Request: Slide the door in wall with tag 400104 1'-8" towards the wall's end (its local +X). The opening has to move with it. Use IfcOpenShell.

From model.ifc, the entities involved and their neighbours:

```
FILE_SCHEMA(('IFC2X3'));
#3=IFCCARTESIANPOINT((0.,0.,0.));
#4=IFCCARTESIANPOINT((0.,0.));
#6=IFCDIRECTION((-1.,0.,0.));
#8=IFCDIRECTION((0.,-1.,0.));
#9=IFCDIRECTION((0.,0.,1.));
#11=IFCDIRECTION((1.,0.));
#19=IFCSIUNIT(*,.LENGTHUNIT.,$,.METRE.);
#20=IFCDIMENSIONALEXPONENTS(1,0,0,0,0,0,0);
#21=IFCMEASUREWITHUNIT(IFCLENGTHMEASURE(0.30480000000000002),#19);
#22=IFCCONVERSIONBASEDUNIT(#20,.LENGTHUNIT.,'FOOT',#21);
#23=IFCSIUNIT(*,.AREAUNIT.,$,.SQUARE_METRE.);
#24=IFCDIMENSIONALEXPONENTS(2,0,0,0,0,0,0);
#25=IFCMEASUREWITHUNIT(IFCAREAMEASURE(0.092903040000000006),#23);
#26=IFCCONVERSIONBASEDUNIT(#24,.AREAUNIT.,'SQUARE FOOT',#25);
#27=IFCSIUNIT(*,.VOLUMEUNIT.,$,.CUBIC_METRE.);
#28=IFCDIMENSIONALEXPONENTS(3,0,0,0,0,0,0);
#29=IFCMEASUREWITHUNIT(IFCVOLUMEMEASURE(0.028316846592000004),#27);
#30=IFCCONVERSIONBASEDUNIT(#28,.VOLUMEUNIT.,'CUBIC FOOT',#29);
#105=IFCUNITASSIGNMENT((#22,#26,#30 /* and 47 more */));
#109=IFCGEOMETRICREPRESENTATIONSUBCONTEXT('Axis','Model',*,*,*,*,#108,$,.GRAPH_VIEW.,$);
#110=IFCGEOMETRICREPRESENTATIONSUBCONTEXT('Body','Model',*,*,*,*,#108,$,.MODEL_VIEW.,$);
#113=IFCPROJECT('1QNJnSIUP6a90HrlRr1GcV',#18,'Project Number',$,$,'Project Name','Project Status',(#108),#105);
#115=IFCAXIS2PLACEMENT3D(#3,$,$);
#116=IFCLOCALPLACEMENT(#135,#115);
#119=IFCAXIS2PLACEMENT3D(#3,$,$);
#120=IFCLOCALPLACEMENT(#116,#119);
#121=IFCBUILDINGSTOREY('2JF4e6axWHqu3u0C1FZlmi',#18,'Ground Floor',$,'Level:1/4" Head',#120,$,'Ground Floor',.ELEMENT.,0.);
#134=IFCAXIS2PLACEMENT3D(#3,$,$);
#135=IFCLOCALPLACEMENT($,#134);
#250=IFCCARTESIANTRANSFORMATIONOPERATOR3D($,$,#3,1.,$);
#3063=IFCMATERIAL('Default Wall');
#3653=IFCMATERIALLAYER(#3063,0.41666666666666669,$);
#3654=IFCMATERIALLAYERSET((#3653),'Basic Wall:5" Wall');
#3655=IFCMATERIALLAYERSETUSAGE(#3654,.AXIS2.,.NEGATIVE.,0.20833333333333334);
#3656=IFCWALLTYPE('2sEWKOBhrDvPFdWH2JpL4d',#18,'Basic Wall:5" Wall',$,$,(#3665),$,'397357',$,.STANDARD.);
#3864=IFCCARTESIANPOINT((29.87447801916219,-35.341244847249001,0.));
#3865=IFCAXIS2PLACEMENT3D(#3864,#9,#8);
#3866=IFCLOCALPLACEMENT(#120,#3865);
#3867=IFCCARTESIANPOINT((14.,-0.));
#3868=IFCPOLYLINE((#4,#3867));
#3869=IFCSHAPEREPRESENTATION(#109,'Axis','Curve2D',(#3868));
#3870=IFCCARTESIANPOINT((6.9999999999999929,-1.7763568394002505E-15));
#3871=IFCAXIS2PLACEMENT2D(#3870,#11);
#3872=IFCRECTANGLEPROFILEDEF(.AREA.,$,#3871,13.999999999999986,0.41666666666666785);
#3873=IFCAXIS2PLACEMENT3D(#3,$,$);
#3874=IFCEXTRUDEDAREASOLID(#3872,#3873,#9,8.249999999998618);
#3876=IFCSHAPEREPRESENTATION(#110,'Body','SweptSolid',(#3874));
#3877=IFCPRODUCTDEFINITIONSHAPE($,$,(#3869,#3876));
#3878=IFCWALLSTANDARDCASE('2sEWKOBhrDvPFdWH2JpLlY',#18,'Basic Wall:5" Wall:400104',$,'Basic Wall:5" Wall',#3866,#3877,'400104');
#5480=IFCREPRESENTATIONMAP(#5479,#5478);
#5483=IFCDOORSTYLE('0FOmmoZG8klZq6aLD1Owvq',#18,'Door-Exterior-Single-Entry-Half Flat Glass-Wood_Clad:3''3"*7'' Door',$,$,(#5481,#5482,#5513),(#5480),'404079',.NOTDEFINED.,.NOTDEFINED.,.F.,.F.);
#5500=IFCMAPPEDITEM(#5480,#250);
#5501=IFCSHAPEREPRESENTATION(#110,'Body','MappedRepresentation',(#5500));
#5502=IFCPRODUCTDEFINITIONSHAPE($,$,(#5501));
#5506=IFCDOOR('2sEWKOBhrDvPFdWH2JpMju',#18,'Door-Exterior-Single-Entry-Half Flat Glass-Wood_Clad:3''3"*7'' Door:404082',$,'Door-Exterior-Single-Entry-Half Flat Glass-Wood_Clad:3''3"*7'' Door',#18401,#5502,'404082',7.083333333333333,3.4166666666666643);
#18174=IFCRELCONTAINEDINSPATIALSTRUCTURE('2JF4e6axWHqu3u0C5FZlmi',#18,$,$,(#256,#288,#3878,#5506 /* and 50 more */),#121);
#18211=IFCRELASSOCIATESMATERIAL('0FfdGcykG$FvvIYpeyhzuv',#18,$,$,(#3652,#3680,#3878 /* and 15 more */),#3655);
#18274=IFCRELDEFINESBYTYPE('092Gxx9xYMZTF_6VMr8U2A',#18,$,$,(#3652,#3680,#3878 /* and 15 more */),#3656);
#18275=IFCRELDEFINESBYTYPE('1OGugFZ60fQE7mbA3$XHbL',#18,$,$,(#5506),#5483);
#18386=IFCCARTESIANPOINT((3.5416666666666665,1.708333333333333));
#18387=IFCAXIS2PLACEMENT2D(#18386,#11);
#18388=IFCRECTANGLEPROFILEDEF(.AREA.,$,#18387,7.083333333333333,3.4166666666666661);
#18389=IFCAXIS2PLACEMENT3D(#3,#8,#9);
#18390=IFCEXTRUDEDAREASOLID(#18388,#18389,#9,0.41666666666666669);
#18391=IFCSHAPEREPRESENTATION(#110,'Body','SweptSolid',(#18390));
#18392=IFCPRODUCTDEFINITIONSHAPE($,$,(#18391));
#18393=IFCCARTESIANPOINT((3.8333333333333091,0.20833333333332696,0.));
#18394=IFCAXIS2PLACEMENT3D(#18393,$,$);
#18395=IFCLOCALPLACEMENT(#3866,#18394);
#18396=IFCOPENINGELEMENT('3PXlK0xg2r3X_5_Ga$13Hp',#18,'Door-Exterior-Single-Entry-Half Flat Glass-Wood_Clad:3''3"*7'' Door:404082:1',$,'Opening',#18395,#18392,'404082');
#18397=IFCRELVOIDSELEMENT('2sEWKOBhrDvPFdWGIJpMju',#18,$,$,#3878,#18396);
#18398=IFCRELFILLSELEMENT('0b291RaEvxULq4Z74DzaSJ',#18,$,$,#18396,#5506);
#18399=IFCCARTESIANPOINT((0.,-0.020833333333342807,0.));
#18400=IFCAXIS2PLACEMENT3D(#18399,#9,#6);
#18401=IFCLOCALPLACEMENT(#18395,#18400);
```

```python
import ifcopenshell
import ifcopenshell.api.geometry
import ifcopenshell.util.placement
import ifcopenshell.util.unit

model = ifcopenshell.open("model.ifc")
unit_scale = ifcopenshell.util.unit.calculate_unit_scale(model)

door = model.by_guid("2sEWKOBhrDvPFdWH2JpMju")
opening = door.FillsVoids[0].RelatingOpeningElement
wall = opening.VoidsElements[0].RelatingBuildingElement

wall_matrix = ifcopenshell.util.placement.get_local_placement(wall.ObjectPlacement)
shift = wall_matrix[:3, 0] * 20 * 0.0254 / unit_scale
before = ifcopenshell.util.placement.get_local_placement(door.ObjectPlacement)[:3, 3].copy()

# The door is placed relative to its opening, so it follows when the opening moves.
matrix = ifcopenshell.util.placement.get_local_placement(opening.ObjectPlacement)
matrix[:3, 3] += shift
ifcopenshell.api.geometry.edit_object_placement(
    model, product=opening, matrix=matrix, is_si=False, should_transform_children=True
)

after = ifcopenshell.util.placement.get_local_placement(door.ObjectPlacement)[:3, 3]
print("door moved by", (after - before).round(3) + 0.0)

model.write("model_updated.ifc")
```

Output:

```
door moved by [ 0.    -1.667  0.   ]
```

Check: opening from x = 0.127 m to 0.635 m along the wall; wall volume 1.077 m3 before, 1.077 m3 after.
